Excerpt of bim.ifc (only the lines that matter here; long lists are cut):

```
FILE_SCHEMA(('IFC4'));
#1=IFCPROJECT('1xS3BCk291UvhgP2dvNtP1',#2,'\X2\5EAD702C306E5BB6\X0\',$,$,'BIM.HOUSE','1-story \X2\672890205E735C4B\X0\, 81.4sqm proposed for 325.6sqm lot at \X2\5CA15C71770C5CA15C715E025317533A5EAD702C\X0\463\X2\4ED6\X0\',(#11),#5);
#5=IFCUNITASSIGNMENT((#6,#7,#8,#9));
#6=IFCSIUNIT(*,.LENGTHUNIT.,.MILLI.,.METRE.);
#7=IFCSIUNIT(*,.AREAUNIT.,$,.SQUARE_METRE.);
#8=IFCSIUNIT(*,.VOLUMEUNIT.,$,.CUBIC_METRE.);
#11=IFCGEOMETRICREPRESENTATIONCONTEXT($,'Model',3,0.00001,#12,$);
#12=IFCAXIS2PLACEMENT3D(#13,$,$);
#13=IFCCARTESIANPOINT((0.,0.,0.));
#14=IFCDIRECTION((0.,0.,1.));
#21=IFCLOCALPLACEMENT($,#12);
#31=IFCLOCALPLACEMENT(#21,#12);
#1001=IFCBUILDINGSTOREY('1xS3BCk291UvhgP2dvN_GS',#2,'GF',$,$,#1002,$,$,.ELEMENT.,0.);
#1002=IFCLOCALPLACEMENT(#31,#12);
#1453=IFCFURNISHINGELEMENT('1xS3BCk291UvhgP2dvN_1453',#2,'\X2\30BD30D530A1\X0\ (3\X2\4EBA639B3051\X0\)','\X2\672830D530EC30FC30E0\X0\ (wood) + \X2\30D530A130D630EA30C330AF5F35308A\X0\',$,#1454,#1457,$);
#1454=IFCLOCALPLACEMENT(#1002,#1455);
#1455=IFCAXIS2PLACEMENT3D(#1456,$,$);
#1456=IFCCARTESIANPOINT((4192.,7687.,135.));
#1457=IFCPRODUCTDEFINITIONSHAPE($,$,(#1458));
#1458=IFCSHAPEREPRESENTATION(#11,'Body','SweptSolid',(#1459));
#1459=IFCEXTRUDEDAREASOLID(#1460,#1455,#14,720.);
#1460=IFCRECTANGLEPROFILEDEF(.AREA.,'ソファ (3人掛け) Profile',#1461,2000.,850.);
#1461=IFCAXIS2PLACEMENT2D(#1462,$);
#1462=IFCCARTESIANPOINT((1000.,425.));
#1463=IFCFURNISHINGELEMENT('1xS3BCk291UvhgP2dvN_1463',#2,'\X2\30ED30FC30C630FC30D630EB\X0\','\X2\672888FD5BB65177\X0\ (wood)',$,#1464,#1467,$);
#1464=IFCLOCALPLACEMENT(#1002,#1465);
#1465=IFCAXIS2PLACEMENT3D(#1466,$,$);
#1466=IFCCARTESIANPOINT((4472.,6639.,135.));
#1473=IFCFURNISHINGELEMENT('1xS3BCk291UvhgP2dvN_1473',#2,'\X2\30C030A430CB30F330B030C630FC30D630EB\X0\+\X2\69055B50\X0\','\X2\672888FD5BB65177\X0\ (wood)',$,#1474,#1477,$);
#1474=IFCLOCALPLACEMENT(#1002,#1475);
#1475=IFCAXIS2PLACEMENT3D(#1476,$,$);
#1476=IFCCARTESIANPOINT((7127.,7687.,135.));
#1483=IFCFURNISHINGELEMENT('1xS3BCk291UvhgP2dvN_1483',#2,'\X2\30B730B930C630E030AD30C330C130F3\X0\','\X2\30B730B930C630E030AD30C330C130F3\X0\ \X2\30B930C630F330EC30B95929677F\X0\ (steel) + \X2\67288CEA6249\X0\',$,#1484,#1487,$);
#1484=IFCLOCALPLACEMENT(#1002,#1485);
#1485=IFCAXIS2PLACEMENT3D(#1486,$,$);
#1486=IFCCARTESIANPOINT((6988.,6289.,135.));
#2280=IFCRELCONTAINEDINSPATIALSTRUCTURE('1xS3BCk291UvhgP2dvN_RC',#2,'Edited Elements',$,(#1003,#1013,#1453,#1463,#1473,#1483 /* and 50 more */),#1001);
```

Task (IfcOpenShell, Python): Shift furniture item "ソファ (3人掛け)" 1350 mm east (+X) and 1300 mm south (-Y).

```python
import ifcopenshell
import ifcopenshell.api.geometry
import ifcopenshell.util.placement
import ifcopenshell.util.unit

model = ifcopenshell.open("bim.ifc")
unit_scale = ifcopenshell.util.unit.calculate_unit_scale(model)

item = model.by_id(1453)
matrix = ifcopenshell.util.placement.get_local_placement(item.ObjectPlacement)
matrix[0, 3] += 1.35 / unit_scale
matrix[1, 3] -= 1.3 / unit_scale
ifcopenshell.api.geometry.edit_object_placement(model, product=item, matrix=matrix, is_si=False)

print(ifcopenshell.util.placement.get_local_placement(item.ObjectPlacement).round(3) + 0.0)

model.write("bim_rev.ifc")
```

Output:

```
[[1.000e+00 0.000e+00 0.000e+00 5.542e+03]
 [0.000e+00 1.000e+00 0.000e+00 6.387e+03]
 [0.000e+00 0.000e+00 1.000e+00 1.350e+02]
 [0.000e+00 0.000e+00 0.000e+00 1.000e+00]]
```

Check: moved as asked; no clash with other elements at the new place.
